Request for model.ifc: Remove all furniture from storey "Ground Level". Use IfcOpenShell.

First a look at what the model holds.

```python
import ifcopenshell
import ifcopenshell.util.element

model = ifcopenshell.open("model.ifc")
print(model.schema)
storey = next(s for s in model.by_type("IfcBuildingStorey") if s.Name == "Ground Level")
furniture = [e for e in ifcopenshell.util.element.get_decomposition(storey) if e.is_a("IfcFurnishingElement")]
seen = {}
for e in furniture:
    element_type = ifcopenshell.util.element.get_type(e)
    name = element_type.Name if element_type not in (None, e) else None
    seen[name] = seen.get(name, 0) + 1
for name, count in sorted(seen.items(), key=str):
    print(count, "x", name)
```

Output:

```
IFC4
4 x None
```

```python
import ifcopenshell
import ifcopenshell.api.root
import ifcopenshell.util.element

model = ifcopenshell.open("model.ifc")

storey = next(s for s in model.by_type("IfcBuildingStorey") if s.Name == "Ground Level")
furniture = [e for e in ifcopenshell.util.element.get_decomposition(storey) if e.is_a("IfcFurnishingElement")]

for e in furniture:
    ifcopenshell.api.root.remove_product(model, product=e)
print(len(furniture), "removed")

model.write("model_edited.ifc")
```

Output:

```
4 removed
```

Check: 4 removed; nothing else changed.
